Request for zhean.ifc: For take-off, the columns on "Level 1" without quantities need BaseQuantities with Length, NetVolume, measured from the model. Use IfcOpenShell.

First a look at what the model holds.

```python
import ifcopenshell
import ifcopenshell.util.element
import ifcopenshell.util.unit

model = ifcopenshell.open("zhean.ifc")
print(model.schema)
for unit_type in ("LENGTHUNIT", "AREAUNIT", "VOLUMEUNIT"):
    print(unit_type, ifcopenshell.util.unit.calculate_unit_scale(model, unit_type))
storey = next(s for s in model.by_type("IfcBuildingStorey") if s.Name == "Level 1")
columns = [e for e in ifcopenshell.util.element.get_decomposition(storey) if e.is_a("IfcColumn")]
for e in sorted(columns, key=lambda e: e.id()):
    print(e.id(), e.is_a(), e.Name, list(ifcopenshell.util.element.get_psets(e, qtos_only=True)), sep=" | ")
```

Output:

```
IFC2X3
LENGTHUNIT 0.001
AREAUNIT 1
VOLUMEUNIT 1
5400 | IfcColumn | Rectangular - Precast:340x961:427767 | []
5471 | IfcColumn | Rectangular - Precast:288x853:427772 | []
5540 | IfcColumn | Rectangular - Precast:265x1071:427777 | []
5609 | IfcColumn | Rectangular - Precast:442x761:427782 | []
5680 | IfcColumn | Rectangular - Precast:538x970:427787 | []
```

```python
import ifcopenshell
import ifcopenshell.api.pset
import ifcopenshell.geom
import ifcopenshell.util.element
import ifcopenshell.util.shape
import ifcopenshell.util.unit

model = ifcopenshell.open("zhean.ifc")
unit_scale = ifcopenshell.util.unit.calculate_unit_scale(model)
volume_scale = ifcopenshell.util.unit.calculate_unit_scale(model, "VOLUMEUNIT")
settings = ifcopenshell.geom.settings()

storey = next(s for s in model.by_type("IfcBuildingStorey") if s.Name == "Level 1")
columns = [e for e in ifcopenshell.util.element.get_decomposition(storey) if e.is_a("IfcColumn")]

for e in sorted(columns, key=lambda e: e.id()):
    if ifcopenshell.util.element.get_psets(e, qtos_only=True, should_inherit=False):
        continue
    # Geometry comes back in metres, in the element's own axes.
    shape = ifcopenshell.geom.create_shape(settings, e)
    values = {
        "Length": ifcopenshell.util.shape.get_z(shape.geometry) / unit_scale,
        "NetVolume": ifcopenshell.util.shape.get_volume(shape.geometry) / volume_scale,
    }
    qto = ifcopenshell.api.pset.add_qto(model, product=e, name="BaseQuantities")
    ifcopenshell.api.pset.edit_qto(model, qto=qto, properties=values)
    print(e.id(), {k: round(v, 3) for k, v in values.items()})

model.write("zhean_rev.ifc")
```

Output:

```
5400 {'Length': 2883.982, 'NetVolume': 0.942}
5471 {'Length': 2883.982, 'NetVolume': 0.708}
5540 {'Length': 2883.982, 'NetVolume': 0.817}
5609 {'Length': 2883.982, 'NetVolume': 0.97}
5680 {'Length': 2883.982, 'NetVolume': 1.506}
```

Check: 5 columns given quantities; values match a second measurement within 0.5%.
